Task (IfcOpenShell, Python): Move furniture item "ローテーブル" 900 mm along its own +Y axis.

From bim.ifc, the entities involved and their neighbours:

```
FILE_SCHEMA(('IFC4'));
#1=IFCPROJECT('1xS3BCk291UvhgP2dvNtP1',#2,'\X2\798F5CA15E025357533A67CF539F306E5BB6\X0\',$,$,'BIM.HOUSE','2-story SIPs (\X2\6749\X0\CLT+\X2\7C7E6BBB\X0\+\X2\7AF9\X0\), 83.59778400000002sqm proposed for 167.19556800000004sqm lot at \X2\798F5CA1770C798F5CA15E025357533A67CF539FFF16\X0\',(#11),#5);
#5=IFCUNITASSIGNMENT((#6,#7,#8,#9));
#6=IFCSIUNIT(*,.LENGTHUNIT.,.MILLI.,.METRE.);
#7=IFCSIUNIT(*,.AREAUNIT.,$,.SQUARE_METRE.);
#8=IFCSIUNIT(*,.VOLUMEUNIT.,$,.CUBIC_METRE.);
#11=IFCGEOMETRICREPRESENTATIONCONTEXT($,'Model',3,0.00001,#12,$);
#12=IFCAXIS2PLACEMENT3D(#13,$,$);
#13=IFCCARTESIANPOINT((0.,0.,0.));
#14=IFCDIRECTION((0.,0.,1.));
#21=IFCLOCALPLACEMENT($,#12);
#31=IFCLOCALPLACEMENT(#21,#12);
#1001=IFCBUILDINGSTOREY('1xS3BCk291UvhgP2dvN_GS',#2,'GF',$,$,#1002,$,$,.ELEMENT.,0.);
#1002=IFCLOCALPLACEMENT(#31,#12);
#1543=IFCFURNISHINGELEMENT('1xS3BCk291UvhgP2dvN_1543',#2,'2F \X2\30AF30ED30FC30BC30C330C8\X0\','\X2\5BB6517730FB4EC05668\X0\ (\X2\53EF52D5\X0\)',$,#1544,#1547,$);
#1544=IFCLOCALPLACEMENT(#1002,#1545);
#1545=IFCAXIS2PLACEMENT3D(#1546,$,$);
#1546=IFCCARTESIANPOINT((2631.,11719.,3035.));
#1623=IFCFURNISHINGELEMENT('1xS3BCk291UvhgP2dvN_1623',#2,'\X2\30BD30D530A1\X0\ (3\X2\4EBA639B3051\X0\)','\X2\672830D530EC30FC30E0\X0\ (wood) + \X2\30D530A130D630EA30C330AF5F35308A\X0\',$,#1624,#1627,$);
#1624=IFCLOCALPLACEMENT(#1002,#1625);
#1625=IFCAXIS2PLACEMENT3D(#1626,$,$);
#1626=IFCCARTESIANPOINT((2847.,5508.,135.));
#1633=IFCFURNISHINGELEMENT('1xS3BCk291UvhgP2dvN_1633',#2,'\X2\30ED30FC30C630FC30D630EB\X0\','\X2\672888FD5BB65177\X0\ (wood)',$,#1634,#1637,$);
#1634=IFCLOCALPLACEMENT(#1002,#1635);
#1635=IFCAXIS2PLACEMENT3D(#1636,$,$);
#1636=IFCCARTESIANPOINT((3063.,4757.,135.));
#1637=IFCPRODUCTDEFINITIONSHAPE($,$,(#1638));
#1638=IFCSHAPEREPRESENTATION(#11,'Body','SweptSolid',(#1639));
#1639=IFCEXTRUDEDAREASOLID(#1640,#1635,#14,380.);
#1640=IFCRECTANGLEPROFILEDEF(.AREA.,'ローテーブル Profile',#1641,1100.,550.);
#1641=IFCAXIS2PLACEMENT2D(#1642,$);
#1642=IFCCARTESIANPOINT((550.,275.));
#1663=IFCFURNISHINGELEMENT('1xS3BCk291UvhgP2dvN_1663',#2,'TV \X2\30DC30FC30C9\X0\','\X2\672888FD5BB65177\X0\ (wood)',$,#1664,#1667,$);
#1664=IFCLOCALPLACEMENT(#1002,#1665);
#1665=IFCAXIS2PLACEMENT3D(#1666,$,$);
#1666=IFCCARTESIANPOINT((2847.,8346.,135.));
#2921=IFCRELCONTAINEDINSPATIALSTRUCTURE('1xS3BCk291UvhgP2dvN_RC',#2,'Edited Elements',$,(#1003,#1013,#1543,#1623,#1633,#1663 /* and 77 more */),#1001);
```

```python
import ifcopenshell
import ifcopenshell.api.geometry
import ifcopenshell.util.placement
import ifcopenshell.util.unit

model = ifcopenshell.open("bim.ifc")
unit_scale = ifcopenshell.util.unit.calculate_unit_scale(model)

item = model.by_id(1633)
matrix = ifcopenshell.util.placement.get_local_placement(item.ObjectPlacement)
matrix[:3, 3] += matrix[:3, 1] * 0.9 / unit_scale
ifcopenshell.api.geometry.edit_object_placement(model, product=item, matrix=matrix, is_si=False)

print(ifcopenshell.util.placement.get_local_placement(item.ObjectPlacement).round(3) + 0.0)

model.write("bim_edited.ifc")
```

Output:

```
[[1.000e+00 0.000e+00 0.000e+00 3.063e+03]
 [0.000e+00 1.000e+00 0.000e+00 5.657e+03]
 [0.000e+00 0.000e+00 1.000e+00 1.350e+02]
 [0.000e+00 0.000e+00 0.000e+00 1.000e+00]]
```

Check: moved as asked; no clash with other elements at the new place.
